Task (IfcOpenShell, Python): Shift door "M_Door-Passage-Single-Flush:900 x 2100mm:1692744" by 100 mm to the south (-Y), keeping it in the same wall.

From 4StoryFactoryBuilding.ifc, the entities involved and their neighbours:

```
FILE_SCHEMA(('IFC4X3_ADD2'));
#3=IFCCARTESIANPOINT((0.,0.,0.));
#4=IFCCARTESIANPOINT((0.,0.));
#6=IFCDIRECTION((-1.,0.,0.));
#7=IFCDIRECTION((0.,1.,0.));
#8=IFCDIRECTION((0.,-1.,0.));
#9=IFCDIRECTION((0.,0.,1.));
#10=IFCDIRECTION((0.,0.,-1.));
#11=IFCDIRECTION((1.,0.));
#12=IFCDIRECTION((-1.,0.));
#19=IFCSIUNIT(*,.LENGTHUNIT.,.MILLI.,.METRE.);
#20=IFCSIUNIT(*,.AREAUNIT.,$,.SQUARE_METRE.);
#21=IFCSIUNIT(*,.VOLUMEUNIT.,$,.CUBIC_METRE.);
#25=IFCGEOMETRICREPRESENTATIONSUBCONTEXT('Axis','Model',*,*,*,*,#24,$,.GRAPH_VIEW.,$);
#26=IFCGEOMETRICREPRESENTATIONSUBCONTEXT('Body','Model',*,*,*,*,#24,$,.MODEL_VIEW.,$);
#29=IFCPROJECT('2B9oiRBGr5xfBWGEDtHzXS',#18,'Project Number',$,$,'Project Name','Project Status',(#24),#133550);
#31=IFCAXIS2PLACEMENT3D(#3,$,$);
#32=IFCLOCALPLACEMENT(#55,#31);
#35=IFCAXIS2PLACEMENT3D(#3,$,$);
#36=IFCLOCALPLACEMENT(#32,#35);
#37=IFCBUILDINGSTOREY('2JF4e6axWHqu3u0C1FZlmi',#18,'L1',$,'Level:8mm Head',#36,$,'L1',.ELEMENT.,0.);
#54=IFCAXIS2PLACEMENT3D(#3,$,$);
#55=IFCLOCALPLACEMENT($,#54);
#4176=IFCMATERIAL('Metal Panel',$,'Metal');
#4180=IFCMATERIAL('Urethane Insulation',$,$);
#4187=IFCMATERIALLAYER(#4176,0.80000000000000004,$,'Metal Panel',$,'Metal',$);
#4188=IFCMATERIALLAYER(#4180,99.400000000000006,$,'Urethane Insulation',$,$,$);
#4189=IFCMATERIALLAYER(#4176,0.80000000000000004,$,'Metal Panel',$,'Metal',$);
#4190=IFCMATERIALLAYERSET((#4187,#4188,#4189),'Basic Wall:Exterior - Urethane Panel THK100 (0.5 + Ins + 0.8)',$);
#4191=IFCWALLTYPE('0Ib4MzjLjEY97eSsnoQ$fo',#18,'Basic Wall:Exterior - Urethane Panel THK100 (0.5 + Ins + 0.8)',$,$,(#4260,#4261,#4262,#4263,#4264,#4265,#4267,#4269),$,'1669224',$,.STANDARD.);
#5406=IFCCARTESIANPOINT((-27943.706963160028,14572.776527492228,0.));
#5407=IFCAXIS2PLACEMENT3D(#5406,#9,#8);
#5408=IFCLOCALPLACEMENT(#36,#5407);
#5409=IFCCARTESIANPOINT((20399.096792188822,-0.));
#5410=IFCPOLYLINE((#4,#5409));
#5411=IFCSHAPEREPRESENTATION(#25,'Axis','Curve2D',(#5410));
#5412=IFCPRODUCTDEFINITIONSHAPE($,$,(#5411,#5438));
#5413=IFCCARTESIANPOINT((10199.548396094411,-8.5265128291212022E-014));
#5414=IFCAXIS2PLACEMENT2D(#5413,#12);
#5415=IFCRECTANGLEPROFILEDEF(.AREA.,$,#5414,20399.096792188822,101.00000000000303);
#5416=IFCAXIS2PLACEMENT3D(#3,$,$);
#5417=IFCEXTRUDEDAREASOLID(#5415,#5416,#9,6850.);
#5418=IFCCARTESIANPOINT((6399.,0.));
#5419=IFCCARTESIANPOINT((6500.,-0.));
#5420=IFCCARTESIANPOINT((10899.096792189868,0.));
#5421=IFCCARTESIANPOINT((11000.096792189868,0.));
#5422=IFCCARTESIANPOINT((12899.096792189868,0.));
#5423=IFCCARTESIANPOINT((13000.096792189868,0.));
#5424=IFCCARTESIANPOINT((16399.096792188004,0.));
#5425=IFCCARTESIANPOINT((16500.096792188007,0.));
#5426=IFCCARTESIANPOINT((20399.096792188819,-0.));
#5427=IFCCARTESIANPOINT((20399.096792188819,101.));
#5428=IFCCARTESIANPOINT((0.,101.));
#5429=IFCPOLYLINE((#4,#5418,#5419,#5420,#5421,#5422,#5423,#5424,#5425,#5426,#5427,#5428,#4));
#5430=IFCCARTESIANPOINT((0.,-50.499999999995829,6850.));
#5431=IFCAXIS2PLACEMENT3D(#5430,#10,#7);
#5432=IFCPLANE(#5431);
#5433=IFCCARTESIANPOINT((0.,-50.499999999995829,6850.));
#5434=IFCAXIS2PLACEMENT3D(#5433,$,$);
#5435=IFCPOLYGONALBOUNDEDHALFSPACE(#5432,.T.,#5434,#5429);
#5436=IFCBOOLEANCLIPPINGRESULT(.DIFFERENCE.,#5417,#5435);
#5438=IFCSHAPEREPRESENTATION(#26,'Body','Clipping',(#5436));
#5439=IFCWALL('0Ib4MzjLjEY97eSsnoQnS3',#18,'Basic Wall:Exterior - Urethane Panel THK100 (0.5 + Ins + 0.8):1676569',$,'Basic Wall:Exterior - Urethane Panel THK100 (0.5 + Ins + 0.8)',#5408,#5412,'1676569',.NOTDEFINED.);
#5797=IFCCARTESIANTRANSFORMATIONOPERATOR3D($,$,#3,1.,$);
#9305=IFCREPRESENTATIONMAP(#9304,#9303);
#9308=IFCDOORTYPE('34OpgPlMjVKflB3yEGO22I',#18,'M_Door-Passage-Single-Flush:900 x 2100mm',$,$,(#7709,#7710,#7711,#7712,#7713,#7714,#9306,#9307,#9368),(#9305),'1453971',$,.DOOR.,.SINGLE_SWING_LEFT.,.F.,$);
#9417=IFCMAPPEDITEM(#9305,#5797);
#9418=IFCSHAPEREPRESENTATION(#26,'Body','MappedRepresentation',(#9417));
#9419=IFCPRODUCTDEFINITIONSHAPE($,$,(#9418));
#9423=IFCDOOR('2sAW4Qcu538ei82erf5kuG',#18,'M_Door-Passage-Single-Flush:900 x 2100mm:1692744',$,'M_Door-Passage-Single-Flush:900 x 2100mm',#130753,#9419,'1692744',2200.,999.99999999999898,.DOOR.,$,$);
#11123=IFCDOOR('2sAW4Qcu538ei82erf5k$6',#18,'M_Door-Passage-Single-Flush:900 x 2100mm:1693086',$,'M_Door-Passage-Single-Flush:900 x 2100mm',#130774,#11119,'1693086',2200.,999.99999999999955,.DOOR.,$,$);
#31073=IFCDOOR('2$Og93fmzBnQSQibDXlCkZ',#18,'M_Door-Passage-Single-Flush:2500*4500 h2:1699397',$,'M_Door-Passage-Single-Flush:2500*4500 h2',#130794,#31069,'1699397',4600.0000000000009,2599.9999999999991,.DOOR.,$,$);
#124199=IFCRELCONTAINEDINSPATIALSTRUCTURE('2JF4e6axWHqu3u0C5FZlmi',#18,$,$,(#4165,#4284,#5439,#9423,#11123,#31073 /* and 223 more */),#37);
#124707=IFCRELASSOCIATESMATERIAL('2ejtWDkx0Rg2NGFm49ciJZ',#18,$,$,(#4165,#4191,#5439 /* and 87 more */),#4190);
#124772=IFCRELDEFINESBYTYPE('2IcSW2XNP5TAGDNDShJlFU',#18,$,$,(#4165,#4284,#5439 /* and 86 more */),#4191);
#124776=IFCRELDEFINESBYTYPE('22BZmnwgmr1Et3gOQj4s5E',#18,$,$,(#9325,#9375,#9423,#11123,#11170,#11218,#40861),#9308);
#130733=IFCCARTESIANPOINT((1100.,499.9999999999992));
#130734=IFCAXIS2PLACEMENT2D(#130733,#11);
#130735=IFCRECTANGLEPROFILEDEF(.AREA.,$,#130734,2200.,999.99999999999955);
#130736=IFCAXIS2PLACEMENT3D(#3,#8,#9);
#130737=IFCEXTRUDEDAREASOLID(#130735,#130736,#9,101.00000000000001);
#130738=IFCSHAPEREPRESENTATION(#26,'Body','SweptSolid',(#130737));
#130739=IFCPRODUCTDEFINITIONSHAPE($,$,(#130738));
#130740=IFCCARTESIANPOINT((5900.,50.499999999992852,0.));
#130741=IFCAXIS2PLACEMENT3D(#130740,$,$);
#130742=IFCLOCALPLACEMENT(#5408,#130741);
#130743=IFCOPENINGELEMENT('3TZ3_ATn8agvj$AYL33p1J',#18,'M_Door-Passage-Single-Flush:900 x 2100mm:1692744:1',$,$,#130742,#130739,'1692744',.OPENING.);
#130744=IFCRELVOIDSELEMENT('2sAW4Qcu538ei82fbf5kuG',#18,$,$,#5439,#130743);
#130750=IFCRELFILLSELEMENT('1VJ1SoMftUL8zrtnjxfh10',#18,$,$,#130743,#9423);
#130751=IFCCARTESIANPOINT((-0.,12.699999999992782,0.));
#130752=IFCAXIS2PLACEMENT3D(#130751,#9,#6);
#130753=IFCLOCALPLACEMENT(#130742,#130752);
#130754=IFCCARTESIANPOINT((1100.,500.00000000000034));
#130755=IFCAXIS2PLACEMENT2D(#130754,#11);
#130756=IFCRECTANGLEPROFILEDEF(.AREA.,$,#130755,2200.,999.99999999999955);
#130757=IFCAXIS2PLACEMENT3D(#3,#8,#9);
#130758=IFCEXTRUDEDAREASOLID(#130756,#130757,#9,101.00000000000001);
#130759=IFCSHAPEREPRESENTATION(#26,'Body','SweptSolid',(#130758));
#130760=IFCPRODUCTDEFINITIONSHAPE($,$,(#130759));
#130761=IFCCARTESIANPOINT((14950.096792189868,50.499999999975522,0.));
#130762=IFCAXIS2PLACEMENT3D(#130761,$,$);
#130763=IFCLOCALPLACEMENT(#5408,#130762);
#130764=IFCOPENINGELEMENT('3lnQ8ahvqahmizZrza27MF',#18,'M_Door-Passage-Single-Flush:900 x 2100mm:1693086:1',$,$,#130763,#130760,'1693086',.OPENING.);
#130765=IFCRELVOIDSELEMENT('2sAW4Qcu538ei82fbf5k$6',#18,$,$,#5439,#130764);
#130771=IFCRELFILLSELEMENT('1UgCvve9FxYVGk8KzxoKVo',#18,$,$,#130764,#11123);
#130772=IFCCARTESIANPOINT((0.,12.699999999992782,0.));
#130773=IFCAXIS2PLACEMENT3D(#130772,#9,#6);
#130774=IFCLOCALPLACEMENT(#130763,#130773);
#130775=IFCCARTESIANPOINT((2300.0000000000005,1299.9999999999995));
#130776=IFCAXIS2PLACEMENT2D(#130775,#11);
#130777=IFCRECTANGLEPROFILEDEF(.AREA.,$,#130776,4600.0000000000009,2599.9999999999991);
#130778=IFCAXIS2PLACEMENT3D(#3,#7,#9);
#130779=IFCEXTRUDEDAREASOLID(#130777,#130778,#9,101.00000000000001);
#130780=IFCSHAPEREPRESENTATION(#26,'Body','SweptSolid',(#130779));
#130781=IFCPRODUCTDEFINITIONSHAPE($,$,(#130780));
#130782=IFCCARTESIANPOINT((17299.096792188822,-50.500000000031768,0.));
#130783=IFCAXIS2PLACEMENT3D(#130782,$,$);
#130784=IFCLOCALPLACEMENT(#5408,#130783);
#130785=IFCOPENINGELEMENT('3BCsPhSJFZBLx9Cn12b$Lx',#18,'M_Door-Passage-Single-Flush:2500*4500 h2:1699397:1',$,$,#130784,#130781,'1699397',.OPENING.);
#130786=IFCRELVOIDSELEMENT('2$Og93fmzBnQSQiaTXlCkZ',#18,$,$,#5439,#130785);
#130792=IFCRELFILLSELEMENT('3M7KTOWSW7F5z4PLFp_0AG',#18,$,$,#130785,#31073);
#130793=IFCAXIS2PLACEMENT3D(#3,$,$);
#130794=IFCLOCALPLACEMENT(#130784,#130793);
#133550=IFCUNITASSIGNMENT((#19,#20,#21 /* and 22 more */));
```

```python
import ifcopenshell
import ifcopenshell.api.geometry
import ifcopenshell.util.placement
import ifcopenshell.util.unit

model = ifcopenshell.open("4StoryFactoryBuilding.ifc")
unit_scale = ifcopenshell.util.unit.calculate_unit_scale(model)

door = model.by_guid("2sAW4Qcu538ei82erf5kuG")
opening = door.FillsVoids[0].RelatingOpeningElement
wall = opening.VoidsElements[0].RelatingBuildingElement

wall_matrix = ifcopenshell.util.placement.get_local_placement(wall.ObjectPlacement)
shift = wall_matrix[:3, 0] * 0.1 / unit_scale
before = ifcopenshell.util.placement.get_local_placement(door.ObjectPlacement)[:3, 3].copy()

# The door is placed relative to its opening, so it follows when the opening moves.
matrix = ifcopenshell.util.placement.get_local_placement(opening.ObjectPlacement)
matrix[:3, 3] += shift
ifcopenshell.api.geometry.edit_object_placement(
    model, product=opening, matrix=matrix, is_si=False, should_transform_children=True
)

after = ifcopenshell.util.placement.get_local_placement(door.ObjectPlacement)[:3, 3]
print("door moved by", (after - before).round(3) + 0.0)

model.write("4StoryFactoryBuilding_v2.ifc")
```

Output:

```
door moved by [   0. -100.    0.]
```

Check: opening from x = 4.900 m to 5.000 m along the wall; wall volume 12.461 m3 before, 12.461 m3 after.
